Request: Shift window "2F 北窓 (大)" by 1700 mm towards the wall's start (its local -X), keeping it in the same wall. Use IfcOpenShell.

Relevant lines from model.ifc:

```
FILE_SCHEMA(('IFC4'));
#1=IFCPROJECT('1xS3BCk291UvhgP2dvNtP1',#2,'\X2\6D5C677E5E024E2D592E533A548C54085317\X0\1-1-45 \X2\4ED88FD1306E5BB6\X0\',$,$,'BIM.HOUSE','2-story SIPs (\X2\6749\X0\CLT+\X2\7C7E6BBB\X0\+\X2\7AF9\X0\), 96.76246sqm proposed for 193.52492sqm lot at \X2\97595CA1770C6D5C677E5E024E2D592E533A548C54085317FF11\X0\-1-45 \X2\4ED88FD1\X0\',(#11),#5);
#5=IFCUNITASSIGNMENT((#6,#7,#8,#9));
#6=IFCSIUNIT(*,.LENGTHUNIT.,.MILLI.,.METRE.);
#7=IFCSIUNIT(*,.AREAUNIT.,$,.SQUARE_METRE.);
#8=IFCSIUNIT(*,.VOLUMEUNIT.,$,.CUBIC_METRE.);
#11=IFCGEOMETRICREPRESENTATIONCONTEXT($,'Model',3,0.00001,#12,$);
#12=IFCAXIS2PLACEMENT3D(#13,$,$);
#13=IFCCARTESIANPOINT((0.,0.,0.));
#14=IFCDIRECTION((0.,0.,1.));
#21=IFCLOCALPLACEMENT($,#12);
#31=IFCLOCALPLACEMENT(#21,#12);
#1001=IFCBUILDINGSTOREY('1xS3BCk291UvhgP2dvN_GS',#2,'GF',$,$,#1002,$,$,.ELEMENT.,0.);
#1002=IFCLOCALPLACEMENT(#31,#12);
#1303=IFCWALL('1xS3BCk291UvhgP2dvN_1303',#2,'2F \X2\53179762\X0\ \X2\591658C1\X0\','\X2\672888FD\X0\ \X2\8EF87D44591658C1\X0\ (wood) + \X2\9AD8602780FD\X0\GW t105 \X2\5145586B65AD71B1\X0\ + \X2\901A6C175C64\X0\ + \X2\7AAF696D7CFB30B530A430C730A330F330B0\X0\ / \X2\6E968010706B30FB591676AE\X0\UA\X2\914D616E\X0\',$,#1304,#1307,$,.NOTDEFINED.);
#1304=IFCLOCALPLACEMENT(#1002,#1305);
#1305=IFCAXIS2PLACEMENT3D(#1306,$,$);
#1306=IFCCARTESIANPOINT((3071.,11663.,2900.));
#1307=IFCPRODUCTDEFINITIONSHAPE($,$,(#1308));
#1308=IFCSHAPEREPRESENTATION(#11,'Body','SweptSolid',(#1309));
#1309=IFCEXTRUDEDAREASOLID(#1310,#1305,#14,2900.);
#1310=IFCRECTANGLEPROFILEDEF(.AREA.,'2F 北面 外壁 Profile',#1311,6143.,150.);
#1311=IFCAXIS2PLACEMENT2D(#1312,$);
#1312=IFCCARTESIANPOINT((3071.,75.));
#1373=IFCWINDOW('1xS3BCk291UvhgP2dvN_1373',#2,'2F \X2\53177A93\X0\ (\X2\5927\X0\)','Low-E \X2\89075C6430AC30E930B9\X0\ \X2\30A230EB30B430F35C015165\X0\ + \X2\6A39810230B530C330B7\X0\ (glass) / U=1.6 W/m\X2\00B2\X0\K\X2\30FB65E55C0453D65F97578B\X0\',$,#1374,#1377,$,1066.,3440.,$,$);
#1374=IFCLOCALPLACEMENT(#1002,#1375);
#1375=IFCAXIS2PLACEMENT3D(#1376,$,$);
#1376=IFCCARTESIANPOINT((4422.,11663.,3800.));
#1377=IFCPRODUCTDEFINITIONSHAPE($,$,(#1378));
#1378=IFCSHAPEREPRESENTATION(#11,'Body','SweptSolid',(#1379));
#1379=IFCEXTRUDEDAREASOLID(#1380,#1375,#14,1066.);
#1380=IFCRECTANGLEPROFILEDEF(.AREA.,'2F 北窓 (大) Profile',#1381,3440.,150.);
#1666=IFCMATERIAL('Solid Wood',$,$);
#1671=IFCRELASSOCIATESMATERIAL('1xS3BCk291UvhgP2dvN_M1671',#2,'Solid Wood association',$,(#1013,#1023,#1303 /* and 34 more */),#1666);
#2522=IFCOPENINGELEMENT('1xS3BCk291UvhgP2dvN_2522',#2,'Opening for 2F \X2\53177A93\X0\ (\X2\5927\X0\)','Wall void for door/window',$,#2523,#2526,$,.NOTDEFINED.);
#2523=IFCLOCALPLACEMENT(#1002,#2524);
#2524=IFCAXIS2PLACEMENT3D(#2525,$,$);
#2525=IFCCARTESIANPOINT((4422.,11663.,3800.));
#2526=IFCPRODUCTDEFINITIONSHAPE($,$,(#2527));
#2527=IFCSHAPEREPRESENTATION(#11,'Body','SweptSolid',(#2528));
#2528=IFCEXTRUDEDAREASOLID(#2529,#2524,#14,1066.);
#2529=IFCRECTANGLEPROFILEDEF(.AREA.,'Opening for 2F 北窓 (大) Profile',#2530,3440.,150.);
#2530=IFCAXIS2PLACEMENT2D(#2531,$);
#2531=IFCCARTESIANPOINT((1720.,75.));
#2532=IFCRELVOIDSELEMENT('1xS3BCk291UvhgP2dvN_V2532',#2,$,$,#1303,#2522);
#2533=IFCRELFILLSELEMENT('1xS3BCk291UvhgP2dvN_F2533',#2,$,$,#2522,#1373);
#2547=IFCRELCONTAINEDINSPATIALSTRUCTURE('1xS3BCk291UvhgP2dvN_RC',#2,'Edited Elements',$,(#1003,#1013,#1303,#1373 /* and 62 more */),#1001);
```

```python
import ifcopenshell
import ifcopenshell.api.geometry
import ifcopenshell.util.placement

model = ifcopenshell.open("model.ifc")

window = model.by_guid("1xS3BCk291UvhgP2dvN_1373")
opening = window.FillsVoids[0].RelatingOpeningElement
wall = opening.VoidsElements[0].RelatingBuildingElement

wall_matrix = ifcopenshell.util.placement.get_local_placement(wall.ObjectPlacement)
shift = wall_matrix[:3, 0] * -1700.0
before = ifcopenshell.util.placement.get_local_placement(window.ObjectPlacement)[:3, 3].copy()

# The window is not placed relative to its opening, so move both.
for product in (opening, window):
    matrix = ifcopenshell.util.placement.get_local_placement(product.ObjectPlacement)
    matrix[:3, 3] += shift
    ifcopenshell.api.geometry.edit_object_placement(model, product=product, matrix=matrix, is_si=False)

after = ifcopenshell.util.placement.get_local_placement(window.ObjectPlacement)[:3, 3]
print("window moved by", (after - before).round(3) + 0.0)

model.write("model_updated.ifc")
```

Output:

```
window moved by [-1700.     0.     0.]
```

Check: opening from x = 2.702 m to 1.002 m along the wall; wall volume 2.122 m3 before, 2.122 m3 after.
